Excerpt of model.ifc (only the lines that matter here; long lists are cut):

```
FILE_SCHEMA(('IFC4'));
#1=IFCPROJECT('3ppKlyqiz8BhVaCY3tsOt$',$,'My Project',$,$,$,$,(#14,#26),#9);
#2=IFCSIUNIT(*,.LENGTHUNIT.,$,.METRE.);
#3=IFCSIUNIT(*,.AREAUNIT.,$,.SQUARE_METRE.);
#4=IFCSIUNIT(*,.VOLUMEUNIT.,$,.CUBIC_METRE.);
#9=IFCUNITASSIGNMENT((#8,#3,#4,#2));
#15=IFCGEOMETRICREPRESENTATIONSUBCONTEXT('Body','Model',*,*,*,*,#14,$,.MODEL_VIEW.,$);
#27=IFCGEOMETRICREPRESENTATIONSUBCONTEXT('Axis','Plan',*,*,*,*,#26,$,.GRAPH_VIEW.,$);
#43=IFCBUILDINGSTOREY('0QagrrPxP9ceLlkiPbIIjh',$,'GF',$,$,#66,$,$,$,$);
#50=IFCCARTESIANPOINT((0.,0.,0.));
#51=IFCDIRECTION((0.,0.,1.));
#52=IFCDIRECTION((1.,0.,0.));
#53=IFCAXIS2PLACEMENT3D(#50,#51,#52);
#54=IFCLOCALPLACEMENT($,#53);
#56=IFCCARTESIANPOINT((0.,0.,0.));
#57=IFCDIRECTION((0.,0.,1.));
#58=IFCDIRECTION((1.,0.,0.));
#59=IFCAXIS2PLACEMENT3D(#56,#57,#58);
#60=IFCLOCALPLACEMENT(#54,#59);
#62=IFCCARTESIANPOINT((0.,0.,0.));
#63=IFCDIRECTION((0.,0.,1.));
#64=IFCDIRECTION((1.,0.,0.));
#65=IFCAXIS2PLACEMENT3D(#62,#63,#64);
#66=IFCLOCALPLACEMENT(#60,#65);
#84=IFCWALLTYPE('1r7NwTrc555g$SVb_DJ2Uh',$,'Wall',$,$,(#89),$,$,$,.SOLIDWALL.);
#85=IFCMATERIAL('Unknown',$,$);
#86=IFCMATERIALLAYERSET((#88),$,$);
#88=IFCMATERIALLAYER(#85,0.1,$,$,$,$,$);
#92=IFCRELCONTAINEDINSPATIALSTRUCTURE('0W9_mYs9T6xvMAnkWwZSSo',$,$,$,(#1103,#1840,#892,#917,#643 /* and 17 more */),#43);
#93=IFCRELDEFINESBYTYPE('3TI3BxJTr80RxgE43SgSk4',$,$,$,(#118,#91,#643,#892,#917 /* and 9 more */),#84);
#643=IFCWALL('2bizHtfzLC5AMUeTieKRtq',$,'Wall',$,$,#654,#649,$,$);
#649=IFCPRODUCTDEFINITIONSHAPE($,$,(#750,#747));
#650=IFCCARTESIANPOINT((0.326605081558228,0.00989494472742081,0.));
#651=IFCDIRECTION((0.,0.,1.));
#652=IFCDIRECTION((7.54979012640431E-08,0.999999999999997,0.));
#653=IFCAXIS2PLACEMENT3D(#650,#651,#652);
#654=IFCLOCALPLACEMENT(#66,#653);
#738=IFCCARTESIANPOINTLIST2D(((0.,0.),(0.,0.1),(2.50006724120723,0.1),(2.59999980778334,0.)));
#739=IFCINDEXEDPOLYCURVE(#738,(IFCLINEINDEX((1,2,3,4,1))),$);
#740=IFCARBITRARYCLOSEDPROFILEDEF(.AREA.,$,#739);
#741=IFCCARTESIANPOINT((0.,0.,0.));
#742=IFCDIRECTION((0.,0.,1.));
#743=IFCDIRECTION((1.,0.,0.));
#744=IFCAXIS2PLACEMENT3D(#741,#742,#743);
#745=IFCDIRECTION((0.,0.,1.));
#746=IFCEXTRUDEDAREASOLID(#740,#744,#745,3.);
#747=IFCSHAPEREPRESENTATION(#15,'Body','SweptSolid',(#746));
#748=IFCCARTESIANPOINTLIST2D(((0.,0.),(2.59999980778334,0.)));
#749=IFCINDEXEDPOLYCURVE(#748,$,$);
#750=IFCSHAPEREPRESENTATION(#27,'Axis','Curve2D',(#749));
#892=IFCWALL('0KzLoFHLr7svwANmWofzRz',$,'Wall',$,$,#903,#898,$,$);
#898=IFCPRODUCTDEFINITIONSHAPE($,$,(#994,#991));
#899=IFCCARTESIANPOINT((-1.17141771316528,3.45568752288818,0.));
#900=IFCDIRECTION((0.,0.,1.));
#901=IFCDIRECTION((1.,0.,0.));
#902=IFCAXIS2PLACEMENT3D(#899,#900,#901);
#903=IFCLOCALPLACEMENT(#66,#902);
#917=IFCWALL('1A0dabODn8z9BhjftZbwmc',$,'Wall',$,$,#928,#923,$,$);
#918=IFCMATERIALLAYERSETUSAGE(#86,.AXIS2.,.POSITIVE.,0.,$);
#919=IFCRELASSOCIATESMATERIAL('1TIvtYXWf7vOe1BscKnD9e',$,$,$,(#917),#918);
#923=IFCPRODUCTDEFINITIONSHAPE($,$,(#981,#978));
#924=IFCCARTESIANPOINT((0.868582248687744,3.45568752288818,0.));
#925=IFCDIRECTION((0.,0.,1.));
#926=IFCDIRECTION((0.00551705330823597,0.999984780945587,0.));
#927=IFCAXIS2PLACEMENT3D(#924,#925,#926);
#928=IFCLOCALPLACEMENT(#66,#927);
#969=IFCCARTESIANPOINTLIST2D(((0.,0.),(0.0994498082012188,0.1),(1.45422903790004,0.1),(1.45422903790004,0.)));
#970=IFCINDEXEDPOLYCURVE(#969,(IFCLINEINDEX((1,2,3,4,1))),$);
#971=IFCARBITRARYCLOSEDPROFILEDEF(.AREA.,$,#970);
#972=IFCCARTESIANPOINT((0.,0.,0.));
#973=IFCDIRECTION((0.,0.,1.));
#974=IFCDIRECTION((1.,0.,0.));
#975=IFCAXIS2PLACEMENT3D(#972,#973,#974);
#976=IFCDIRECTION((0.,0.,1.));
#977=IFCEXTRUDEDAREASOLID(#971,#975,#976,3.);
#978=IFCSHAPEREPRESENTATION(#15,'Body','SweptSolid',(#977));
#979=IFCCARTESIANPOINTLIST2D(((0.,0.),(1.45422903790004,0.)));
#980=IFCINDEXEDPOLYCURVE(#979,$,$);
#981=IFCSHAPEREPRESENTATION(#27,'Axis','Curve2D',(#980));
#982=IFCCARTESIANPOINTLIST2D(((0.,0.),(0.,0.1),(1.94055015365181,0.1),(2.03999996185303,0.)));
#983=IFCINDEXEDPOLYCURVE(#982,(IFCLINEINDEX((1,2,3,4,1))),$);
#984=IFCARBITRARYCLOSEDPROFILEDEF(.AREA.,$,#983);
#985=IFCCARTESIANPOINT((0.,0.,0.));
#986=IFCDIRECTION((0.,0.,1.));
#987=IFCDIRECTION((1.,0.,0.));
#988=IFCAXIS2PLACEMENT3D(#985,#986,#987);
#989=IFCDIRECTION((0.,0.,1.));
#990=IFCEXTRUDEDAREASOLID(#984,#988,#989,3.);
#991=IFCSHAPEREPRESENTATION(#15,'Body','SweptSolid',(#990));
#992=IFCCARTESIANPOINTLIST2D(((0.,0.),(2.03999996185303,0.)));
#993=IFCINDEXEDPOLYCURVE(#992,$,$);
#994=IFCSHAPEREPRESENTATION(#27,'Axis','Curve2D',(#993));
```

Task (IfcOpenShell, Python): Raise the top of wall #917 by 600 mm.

```python
import ifcopenshell
import ifcopenshell.geom
import ifcopenshell.util.representation
import ifcopenshell.util.shape
import ifcopenshell.util.unit

model = ifcopenshell.open("model.ifc")
unit_scale = ifcopenshell.util.unit.calculate_unit_scale(model)
settings = ifcopenshell.geom.settings()


def volume(element):
    """Net volume in cubic metres, openings subtracted."""
    shape = ifcopenshell.geom.create_shape(settings, element)
    return ifcopenshell.util.shape.get_volume(shape.geometry)


wall = model.by_guid("1A0dabODn8z9BhjftZbwmc")
before = volume(wall)

body = ifcopenshell.util.representation.get_representation(wall, "Model", "Body")
solid = body.Items[0]
old_height = solid.Depth
solid.Depth += 0.6 / unit_scale
after = volume(wall)

print(f"height {old_height:g} -> {solid.Depth:g}, volume {before:.3f} -> {after:.3f} m3")

model.write("model-out.ifc")
```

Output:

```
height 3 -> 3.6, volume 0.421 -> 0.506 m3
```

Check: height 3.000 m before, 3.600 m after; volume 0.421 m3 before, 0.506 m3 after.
